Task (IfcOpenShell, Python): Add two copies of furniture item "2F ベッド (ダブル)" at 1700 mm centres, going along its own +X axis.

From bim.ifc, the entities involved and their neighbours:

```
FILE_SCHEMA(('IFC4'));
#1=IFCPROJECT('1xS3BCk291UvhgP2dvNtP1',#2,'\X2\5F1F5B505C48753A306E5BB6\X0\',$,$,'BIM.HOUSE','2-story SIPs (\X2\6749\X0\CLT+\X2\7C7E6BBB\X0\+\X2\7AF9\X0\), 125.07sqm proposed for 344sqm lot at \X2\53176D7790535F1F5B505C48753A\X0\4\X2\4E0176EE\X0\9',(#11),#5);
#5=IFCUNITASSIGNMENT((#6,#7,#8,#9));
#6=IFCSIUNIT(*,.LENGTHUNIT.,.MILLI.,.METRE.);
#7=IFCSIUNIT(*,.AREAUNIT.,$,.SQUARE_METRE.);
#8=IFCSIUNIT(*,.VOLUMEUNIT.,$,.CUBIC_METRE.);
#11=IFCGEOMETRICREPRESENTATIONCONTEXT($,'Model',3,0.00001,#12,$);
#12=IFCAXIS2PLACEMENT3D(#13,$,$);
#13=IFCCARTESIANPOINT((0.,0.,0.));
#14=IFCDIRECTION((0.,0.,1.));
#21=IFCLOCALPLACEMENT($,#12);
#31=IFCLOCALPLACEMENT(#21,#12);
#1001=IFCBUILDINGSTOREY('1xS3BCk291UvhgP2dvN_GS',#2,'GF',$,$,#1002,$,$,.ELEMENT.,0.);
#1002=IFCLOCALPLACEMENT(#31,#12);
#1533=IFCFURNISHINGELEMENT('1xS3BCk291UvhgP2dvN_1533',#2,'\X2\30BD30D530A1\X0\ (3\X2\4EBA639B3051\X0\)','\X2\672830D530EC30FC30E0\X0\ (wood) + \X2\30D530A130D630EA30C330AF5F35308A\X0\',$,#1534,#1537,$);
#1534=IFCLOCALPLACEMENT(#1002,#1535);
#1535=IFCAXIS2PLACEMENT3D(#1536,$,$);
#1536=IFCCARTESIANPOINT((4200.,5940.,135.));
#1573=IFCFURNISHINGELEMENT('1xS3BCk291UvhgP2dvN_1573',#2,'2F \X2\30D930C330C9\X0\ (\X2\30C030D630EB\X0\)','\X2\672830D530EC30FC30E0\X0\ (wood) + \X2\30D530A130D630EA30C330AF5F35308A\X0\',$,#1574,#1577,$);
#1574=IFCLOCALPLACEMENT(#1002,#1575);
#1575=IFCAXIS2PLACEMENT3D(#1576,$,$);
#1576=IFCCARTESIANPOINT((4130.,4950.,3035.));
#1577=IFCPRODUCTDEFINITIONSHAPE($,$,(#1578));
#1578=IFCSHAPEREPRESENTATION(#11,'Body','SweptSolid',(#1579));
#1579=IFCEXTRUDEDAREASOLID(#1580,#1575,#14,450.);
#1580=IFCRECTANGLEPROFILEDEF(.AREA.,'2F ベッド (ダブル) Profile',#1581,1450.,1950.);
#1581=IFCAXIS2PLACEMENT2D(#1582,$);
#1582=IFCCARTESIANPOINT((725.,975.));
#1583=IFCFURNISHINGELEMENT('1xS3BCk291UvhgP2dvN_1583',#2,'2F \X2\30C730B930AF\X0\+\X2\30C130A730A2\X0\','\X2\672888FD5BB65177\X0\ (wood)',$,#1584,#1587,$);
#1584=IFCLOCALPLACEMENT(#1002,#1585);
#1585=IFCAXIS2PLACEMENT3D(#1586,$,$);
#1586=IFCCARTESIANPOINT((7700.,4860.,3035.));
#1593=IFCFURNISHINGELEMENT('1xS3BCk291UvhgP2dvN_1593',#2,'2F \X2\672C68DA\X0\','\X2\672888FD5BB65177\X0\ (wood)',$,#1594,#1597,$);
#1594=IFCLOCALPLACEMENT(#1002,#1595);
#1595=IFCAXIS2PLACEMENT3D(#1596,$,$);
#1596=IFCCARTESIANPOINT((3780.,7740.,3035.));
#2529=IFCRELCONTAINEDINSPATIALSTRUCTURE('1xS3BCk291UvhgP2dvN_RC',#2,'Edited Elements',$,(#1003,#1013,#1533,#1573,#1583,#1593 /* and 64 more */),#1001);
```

```python
import ifcopenshell
import ifcopenshell.api.geometry
import ifcopenshell.api.root
import ifcopenshell.util.element
import ifcopenshell.util.placement

model = ifcopenshell.open("bim.ifc")


def reuse_history(source, copy):
    """copy_class also copies each property set's owner history, people and application; keep the originals."""
    for rel in copy.IsDefinedBy:
        if rel.is_a("IfcRelDefinesByProperties") and (history := rel.RelatingPropertyDefinition.OwnerHistory):
            rel.RelatingPropertyDefinition.OwnerHistory = source.OwnerHistory
            ifcopenshell.util.element.remove_deep2(model, history)


source = model.by_id(1573)
base = ifcopenshell.util.placement.get_local_placement(source.ObjectPlacement)
step = base[:3, 0] * 1700.0

for i in range(1, 3):
    copy = ifcopenshell.api.root.copy_class(model, product=source)
    copy.Representation = ifcopenshell.util.element.copy_deep(
        model, source.Representation, exclude=["IfcGeometricRepresentationContext", "IfcRepresentationMap"]
    )
    reuse_history(source, copy)
    matrix = base.copy()
    matrix[:3, 3] += i * step
    print("added at", matrix[:3, 3].round(3) + 0.0)
    ifcopenshell.api.geometry.edit_object_placement(model, product=copy, matrix=matrix, is_si=False)

model.write("bim_v2.ifc")
```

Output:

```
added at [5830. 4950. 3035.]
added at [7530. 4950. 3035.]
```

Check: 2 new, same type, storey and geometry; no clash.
